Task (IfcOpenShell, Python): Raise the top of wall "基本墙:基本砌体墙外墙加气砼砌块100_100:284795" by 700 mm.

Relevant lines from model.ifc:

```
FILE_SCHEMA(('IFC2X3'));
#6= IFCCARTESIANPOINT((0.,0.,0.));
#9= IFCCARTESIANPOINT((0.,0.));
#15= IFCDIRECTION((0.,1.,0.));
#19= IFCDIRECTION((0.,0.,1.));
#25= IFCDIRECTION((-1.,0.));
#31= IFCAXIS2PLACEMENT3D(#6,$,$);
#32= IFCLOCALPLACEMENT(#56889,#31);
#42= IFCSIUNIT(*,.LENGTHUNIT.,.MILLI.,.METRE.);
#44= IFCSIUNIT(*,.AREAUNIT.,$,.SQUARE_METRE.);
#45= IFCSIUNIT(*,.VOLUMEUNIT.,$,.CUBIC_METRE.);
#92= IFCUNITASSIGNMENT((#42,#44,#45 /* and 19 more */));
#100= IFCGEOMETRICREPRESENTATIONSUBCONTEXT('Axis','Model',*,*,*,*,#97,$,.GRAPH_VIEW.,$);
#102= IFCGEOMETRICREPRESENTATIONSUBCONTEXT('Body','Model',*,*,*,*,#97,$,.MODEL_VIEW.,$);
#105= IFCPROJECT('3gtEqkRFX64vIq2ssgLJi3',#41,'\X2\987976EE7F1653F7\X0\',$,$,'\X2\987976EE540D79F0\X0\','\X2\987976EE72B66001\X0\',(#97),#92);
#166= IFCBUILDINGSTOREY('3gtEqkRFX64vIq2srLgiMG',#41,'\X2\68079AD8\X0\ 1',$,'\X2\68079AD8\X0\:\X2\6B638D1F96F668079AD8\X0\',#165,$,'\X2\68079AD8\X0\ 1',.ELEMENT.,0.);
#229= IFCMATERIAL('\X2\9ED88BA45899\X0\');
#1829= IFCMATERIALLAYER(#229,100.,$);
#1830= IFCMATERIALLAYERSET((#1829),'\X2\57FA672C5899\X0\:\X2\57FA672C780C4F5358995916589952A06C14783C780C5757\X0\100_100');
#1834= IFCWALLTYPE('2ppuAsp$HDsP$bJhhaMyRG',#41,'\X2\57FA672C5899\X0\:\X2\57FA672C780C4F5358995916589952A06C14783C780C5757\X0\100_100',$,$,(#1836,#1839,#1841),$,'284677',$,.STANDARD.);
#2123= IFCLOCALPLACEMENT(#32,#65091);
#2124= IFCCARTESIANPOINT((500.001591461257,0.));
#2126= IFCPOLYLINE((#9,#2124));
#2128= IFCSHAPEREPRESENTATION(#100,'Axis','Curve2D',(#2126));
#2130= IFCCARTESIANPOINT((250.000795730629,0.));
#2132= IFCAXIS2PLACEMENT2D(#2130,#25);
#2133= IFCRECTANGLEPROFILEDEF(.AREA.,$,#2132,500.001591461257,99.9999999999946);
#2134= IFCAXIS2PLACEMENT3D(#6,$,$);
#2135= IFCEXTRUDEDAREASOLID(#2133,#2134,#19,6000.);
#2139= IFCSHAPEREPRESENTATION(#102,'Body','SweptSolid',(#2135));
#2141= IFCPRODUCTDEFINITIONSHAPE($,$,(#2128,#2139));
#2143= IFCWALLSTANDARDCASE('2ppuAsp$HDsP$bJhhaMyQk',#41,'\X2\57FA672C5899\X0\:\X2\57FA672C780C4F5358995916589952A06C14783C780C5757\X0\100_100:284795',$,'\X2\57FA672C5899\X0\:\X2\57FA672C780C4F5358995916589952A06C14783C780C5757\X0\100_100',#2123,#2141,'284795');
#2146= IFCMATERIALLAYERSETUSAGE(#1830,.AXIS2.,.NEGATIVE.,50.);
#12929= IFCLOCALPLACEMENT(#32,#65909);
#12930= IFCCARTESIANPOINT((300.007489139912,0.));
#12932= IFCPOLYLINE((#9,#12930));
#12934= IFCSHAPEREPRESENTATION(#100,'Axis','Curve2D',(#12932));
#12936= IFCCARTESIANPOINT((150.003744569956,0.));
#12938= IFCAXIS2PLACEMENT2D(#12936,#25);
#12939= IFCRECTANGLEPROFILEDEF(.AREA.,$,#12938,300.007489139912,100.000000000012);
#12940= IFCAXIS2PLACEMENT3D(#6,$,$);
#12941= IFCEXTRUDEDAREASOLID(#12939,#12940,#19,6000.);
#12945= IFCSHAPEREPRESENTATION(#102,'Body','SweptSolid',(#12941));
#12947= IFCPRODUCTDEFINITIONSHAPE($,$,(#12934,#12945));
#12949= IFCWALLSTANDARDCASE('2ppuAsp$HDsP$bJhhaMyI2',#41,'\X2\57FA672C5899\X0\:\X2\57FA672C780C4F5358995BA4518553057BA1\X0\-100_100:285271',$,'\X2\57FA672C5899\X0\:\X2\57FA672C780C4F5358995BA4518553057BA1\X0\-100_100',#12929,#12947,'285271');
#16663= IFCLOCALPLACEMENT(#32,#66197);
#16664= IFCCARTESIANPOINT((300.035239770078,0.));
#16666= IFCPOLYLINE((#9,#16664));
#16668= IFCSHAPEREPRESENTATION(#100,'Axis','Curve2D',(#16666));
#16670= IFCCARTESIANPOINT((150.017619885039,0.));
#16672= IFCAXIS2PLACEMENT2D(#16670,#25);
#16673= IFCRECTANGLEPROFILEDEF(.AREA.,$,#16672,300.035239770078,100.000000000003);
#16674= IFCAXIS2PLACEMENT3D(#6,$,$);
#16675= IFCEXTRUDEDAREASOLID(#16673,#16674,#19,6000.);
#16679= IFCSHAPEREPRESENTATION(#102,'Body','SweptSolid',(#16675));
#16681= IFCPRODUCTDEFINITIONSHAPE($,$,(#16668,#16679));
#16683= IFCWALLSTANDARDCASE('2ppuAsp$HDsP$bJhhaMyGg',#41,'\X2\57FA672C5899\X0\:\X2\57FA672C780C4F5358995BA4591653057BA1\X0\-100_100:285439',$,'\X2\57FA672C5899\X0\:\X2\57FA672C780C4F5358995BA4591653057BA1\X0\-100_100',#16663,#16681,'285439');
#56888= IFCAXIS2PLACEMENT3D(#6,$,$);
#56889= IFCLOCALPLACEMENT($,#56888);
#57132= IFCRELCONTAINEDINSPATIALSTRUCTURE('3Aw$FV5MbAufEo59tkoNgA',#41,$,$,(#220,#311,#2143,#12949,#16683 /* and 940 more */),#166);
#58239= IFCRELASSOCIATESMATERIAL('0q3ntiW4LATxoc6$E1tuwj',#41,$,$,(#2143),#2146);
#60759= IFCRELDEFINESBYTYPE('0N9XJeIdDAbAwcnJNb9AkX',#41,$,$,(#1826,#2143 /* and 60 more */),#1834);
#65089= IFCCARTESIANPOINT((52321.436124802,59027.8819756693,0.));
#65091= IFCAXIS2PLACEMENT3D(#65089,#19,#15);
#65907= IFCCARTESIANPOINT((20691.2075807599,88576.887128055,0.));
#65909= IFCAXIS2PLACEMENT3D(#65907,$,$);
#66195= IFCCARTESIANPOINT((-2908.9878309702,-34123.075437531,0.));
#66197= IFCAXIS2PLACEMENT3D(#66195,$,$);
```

```python
import ifcopenshell
import ifcopenshell.geom
import ifcopenshell.util.representation
import ifcopenshell.util.shape
import ifcopenshell.util.unit

model = ifcopenshell.open("model.ifc")
unit_scale = ifcopenshell.util.unit.calculate_unit_scale(model)
settings = ifcopenshell.geom.settings()


def volume(element):
    """Net volume in cubic metres, openings subtracted."""
    shape = ifcopenshell.geom.create_shape(settings, element)
    return ifcopenshell.util.shape.get_volume(shape.geometry)


wall = model.by_guid("2ppuAsp$HDsP$bJhhaMyQk")
before = volume(wall)

body = ifcopenshell.util.representation.get_representation(wall, "Model", "Body")
solid = body.Items[0]
old_height = solid.Depth
solid.Depth += 0.7 / unit_scale
after = volume(wall)

print(f"height {old_height:g} -> {solid.Depth:g}, volume {before:.3f} -> {after:.3f} m3")

model.write("model-out.ifc")
```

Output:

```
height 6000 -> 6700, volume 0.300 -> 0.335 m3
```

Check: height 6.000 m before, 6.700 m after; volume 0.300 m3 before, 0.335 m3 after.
